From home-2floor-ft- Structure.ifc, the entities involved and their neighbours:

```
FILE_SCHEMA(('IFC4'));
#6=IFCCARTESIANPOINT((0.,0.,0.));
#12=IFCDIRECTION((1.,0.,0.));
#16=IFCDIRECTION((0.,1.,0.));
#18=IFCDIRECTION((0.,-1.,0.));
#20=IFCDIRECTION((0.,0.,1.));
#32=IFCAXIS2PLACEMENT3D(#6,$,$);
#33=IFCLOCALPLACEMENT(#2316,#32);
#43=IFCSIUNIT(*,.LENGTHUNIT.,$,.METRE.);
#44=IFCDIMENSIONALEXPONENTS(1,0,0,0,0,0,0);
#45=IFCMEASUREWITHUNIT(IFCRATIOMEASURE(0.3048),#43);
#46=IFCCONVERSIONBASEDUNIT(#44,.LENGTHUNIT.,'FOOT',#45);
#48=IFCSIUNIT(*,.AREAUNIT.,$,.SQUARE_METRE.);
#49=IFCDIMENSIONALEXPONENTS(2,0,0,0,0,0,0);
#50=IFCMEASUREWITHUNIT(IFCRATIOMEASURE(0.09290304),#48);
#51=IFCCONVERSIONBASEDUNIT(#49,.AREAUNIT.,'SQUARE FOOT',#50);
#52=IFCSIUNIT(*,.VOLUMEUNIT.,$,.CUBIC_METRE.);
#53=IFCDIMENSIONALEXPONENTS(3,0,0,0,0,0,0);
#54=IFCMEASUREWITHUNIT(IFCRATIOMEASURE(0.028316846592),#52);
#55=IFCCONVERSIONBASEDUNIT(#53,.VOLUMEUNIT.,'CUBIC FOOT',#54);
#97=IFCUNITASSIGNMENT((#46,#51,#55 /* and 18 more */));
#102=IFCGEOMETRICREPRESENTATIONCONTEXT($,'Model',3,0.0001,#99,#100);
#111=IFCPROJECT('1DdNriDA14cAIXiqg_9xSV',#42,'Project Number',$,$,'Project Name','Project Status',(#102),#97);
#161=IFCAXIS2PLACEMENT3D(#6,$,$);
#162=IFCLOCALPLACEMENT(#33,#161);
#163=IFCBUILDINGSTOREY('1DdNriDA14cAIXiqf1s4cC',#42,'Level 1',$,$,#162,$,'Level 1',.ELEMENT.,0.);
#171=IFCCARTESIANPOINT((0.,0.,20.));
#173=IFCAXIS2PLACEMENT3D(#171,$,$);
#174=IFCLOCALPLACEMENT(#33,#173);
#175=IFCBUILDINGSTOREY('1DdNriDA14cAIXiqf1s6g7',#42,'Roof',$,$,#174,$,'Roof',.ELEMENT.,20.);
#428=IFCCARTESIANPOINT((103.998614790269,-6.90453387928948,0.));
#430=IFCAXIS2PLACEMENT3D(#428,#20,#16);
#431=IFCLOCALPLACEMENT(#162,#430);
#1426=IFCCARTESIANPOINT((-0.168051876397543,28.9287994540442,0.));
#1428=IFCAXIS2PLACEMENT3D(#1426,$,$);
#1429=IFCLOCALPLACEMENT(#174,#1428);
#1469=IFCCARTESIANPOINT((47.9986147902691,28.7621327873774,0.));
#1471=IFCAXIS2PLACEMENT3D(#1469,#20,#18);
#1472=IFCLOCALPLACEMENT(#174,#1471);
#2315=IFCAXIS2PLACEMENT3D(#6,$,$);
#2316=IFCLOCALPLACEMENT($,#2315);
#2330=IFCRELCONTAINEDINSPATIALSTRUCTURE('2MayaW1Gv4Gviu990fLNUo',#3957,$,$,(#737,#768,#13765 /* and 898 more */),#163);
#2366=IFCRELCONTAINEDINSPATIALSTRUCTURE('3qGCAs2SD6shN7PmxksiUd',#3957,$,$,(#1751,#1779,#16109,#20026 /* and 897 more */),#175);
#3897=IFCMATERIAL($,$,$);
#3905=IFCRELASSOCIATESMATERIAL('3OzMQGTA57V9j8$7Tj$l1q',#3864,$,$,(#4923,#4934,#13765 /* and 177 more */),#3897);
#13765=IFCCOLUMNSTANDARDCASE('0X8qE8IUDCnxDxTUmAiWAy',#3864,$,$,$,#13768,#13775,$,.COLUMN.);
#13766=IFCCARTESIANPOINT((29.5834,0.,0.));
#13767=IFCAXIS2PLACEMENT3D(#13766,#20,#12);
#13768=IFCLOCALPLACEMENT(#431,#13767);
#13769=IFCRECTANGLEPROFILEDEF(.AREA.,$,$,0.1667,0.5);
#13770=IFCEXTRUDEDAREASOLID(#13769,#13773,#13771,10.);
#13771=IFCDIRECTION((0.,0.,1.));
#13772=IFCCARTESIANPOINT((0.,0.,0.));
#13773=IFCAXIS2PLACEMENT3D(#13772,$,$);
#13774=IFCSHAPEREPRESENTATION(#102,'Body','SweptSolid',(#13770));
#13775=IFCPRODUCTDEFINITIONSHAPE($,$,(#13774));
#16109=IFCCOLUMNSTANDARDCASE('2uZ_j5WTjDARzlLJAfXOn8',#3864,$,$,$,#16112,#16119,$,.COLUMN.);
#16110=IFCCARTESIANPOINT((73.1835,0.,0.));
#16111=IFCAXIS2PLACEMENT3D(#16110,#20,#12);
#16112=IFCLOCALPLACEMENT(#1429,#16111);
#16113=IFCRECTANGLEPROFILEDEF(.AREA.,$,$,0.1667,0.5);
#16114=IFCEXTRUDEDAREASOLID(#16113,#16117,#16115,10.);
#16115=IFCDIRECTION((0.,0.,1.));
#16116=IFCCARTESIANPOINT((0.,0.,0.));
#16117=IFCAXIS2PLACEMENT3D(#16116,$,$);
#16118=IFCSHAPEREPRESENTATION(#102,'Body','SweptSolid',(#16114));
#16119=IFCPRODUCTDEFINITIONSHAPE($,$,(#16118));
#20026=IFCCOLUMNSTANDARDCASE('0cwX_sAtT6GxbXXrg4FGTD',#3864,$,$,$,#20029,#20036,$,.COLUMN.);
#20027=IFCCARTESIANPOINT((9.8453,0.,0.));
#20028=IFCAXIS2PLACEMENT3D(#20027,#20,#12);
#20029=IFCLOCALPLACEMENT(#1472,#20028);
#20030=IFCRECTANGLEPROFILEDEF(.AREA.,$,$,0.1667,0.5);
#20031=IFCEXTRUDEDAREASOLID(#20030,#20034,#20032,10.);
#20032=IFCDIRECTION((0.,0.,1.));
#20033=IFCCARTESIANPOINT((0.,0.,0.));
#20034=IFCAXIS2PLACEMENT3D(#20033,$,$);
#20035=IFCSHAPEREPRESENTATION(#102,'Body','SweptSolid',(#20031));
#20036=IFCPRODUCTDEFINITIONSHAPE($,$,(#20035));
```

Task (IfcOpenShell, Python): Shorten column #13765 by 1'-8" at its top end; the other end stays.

```python
import ifcopenshell
import ifcopenshell.util.unit

model = ifcopenshell.open("home-2floor-ft- Structure.ifc")
unit_scale = ifcopenshell.util.unit.calculate_unit_scale(model)

member = model.by_guid("0X8qE8IUDCnxDxTUmAiWAy")
change = -20 * 0.0254 / unit_scale

# The extrusion runs towards the end named, so only its depth changes.
body = next(r for r in member.Representation.Representations if r.RepresentationIdentifier == "Body")
solid = body.Items[0]
old_length = solid.Depth
solid.Depth += change

print(f"length {old_length:g} -> {solid.Depth:g}")

model.write("home-2floor-ft- Structure_rev.ifc")
```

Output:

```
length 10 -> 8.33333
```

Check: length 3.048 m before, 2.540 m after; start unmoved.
